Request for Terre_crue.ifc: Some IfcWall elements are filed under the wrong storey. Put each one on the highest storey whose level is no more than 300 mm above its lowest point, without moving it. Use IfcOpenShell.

First a look at what the model holds.

```python
import ifcopenshell
import ifcopenshell.util.element
import ifcopenshell.util.placement

model = ifcopenshell.open("Terre_crue.ifc")
print(model.schema)
for storey in model.by_type("IfcBuildingStorey"):
    level = ifcopenshell.util.placement.get_storey_elevation(storey)
    count = sum(e.is_a("IfcWall") for e in ifcopenshell.util.element.get_contained(storey))
    print(storey.id(), storey.Name, round(level, 3), count, sep=" | ")
```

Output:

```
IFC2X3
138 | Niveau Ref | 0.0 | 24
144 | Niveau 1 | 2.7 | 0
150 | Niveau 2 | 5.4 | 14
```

```python
import ifcopenshell
import ifcopenshell.api.spatial
import ifcopenshell.geom
import ifcopenshell.util.element
import ifcopenshell.util.placement
import ifcopenshell.util.shape
import ifcopenshell.util.unit

model = ifcopenshell.open("Terre_crue.ifc")
unit_scale = ifcopenshell.util.unit.calculate_unit_scale(model)
settings = ifcopenshell.geom.settings()

levels = sorted(
    ((ifcopenshell.util.placement.get_storey_elevation(s) * unit_scale, s) for s in model.by_type("IfcBuildingStorey")),
    key=lambda pair: pair[0],
)

for e in model.by_type("IfcWall"):
    current = e.ContainedInStructure[0].RelatingStructure if e.ContainedInStructure else None
    if current is None or not current.is_a("IfcBuildingStorey"):
        continue
    shape = ifcopenshell.geom.create_shape(settings, e)
    bottom = ifcopenshell.util.shape.get_shape_bottom_elevation(shape, shape.geometry)
    below = [s for level, s in levels if level <= bottom + 0.3]
    storey = below[-1] if below else levels[0][1]
    if storey != current:
        # assign_container keeps the world position.
        ifcopenshell.api.spatial.assign_container(model, products=[e], relating_structure=storey)
        print(e.id(), current.Name, "->", storey.Name)

model.write("Terre_crue_edited.ifc")
```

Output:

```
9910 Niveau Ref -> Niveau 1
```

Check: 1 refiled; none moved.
